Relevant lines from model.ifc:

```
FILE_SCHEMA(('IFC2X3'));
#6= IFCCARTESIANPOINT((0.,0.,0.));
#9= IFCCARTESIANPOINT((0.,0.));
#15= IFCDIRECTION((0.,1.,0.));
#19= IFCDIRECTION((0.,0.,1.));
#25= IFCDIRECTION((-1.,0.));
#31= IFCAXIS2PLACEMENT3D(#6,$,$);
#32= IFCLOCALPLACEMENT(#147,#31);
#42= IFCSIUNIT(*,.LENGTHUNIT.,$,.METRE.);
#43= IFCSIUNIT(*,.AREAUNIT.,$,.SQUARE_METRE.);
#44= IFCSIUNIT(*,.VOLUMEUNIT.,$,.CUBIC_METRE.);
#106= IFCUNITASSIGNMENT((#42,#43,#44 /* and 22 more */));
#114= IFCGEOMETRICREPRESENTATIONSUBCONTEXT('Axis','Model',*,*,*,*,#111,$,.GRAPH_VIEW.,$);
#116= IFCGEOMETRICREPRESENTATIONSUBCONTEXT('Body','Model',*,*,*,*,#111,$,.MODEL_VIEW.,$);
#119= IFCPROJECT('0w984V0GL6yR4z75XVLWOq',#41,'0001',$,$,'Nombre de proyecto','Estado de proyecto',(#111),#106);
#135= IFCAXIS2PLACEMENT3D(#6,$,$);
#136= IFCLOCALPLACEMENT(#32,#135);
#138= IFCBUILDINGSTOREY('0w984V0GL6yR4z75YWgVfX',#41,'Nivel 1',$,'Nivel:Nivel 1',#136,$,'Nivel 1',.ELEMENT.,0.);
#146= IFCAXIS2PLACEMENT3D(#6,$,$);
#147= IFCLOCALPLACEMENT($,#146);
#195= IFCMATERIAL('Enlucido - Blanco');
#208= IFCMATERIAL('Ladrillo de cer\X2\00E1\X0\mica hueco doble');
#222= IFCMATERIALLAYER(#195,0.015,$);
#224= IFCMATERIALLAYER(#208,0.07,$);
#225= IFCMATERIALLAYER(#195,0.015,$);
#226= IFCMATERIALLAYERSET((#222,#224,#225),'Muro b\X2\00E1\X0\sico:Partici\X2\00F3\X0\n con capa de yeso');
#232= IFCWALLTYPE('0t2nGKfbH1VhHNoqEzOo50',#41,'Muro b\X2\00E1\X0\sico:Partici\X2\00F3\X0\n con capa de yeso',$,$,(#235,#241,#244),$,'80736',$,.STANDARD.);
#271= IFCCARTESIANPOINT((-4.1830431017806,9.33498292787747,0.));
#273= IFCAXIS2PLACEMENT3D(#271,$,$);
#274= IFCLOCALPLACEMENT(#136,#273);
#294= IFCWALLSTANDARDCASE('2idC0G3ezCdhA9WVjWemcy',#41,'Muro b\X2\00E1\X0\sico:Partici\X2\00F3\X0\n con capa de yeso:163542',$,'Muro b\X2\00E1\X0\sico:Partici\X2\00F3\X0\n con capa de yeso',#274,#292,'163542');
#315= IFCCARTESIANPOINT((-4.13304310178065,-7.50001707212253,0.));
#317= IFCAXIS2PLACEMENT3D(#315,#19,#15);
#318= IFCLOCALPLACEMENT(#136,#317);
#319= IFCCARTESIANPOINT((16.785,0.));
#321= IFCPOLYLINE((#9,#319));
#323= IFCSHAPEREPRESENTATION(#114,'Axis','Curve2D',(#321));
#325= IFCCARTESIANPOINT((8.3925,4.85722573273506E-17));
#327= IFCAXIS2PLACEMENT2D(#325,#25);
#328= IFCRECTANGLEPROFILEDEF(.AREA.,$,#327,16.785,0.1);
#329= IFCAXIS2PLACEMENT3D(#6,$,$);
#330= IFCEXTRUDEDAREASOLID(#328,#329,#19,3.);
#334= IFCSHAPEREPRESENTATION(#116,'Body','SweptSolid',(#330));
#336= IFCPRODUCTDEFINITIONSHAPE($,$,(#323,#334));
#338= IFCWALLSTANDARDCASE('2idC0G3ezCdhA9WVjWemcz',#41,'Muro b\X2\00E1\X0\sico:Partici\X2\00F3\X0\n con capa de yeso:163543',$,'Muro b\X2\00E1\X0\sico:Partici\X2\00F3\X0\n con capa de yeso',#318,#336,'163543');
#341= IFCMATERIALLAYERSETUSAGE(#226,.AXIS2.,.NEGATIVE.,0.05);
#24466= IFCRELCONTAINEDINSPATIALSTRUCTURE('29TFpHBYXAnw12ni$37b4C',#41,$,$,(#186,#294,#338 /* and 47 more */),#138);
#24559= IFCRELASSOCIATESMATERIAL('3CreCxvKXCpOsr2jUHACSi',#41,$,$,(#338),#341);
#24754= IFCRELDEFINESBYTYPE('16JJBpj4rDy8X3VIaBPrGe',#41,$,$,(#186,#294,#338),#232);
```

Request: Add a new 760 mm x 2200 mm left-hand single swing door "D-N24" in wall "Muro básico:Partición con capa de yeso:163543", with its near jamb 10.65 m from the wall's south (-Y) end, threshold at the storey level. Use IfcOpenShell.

```python
import numpy as np
import ifcopenshell
import ifcopenshell.api.feature
import ifcopenshell.api.geometry
import ifcopenshell.api.root
import ifcopenshell.api.spatial
import ifcopenshell.api.type
import ifcopenshell.geom
import ifcopenshell.util.element
import ifcopenshell.util.placement
import ifcopenshell.util.representation
import ifcopenshell.util.shape
import ifcopenshell.util.unit

model = ifcopenshell.open("model.ifc")
unit_scale = ifcopenshell.util.unit.calculate_unit_scale(model)
settings = ifcopenshell.geom.settings()


def volume(element):
    """Net volume in cubic metres, openings subtracted."""
    shape = ifcopenshell.geom.create_shape(settings, element)
    return ifcopenshell.util.shape.get_volume(shape.geometry)


wall = model.by_guid("2idC0G3ezCdhA9WVjWemcz")
storey = ifcopenshell.util.element.get_container(wall, ifc_class="IfcBuildingStorey")
context = ifcopenshell.util.representation.get_context(model, "Model", "Body", "MODEL_VIEW")
before = volume(wall)

width, height, from_end, sill = 0.76, 2.2, 10.65, 0.0  # metres

# The wall runs along its own X axis, and the end named is its -X end.
wall_shape = ifcopenshell.geom.create_shape(settings, wall)
x, y, z = ifcopenshell.util.shape.get_vertices(wall_shape.geometry).T
start = x.min() + from_end
face, thickness = float(y.min()), float(y.max() - y.min())
wall_matrix = ifcopenshell.util.placement.get_local_placement(wall.ObjectPlacement)
level = ifcopenshell.util.placement.get_local_placement(storey.ObjectPlacement)[2, 3]


def in_wall(x, y):
    """Placement at x, y metres in the wall's axes, at sill height."""
    matrix = wall_matrix.copy()
    matrix[:, 3] = wall_matrix @ np.array([x / unit_scale, y / unit_scale, 0.0, 1.0])
    matrix[2, 3] = level + sill / unit_scale
    return matrix


# Opening: a box that overshoots both wall faces by 50 mm.
opening = ifcopenshell.api.root.create_entity(model, ifc_class="IfcOpeningElement")
box = ifcopenshell.api.geometry.add_wall_representation(
    model, context=context, length=width, height=height, thickness=thickness + 0.1
)
ifcopenshell.api.geometry.assign_representation(model, product=opening, representation=box)
ifcopenshell.api.geometry.edit_object_placement(model, product=opening, matrix=in_wall(start, face - 0.05), is_si=False)
ifcopenshell.api.feature.add_feature(model, feature=opening, element=wall)

door = ifcopenshell.api.root.create_entity(model, ifc_class="IfcDoor", name="D-N24")
door.OverallWidth, door.OverallHeight = width / unit_scale, height / unit_scale
body = ifcopenshell.api.geometry.add_door_representation(
    model,
    context=context,
    overall_width=door.OverallWidth,
    overall_height=door.OverallHeight,
    operation_type="SINGLE_SWING_LEFT",
    lining_properties={"LiningDepth": thickness / unit_scale, "ThresholdDepth": thickness / unit_scale},
)
ifcopenshell.api.geometry.assign_representation(model, product=door, representation=body)
ifcopenshell.api.spatial.assign_container(model, products=[door], relating_structure=storey)
fills = ifcopenshell.api.feature.add_filling(model, opening=opening, element=door)
fills.OwnerHistory = door.OwnerHistory  # required in IFC2X3

# IFC2X3 keeps the operation on the door style.
style = ifcopenshell.api.root.create_entity(model, ifc_class="IfcDoorStyle", name="D-N24")
style.OperationType, style.ConstructionType = "SINGLE_SWING_LEFT", "NOTDEFINED"
style.ParameterTakesPrecedence = style.Sizeable = False
ifcopenshell.api.type.assign_type(model, related_objects=[door], relating_type=style)

# The lining spans the wall, so the door starts at the wall face.
ifcopenshell.api.geometry.edit_object_placement(model, product=door, matrix=in_wall(start, face), is_si=False)

after = volume(wall)

print(f"wall volume {before:.3f} -> {after:.3f} m3")

model.write("model_updated.ifc")
```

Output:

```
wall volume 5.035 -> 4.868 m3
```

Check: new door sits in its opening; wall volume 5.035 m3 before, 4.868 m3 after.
